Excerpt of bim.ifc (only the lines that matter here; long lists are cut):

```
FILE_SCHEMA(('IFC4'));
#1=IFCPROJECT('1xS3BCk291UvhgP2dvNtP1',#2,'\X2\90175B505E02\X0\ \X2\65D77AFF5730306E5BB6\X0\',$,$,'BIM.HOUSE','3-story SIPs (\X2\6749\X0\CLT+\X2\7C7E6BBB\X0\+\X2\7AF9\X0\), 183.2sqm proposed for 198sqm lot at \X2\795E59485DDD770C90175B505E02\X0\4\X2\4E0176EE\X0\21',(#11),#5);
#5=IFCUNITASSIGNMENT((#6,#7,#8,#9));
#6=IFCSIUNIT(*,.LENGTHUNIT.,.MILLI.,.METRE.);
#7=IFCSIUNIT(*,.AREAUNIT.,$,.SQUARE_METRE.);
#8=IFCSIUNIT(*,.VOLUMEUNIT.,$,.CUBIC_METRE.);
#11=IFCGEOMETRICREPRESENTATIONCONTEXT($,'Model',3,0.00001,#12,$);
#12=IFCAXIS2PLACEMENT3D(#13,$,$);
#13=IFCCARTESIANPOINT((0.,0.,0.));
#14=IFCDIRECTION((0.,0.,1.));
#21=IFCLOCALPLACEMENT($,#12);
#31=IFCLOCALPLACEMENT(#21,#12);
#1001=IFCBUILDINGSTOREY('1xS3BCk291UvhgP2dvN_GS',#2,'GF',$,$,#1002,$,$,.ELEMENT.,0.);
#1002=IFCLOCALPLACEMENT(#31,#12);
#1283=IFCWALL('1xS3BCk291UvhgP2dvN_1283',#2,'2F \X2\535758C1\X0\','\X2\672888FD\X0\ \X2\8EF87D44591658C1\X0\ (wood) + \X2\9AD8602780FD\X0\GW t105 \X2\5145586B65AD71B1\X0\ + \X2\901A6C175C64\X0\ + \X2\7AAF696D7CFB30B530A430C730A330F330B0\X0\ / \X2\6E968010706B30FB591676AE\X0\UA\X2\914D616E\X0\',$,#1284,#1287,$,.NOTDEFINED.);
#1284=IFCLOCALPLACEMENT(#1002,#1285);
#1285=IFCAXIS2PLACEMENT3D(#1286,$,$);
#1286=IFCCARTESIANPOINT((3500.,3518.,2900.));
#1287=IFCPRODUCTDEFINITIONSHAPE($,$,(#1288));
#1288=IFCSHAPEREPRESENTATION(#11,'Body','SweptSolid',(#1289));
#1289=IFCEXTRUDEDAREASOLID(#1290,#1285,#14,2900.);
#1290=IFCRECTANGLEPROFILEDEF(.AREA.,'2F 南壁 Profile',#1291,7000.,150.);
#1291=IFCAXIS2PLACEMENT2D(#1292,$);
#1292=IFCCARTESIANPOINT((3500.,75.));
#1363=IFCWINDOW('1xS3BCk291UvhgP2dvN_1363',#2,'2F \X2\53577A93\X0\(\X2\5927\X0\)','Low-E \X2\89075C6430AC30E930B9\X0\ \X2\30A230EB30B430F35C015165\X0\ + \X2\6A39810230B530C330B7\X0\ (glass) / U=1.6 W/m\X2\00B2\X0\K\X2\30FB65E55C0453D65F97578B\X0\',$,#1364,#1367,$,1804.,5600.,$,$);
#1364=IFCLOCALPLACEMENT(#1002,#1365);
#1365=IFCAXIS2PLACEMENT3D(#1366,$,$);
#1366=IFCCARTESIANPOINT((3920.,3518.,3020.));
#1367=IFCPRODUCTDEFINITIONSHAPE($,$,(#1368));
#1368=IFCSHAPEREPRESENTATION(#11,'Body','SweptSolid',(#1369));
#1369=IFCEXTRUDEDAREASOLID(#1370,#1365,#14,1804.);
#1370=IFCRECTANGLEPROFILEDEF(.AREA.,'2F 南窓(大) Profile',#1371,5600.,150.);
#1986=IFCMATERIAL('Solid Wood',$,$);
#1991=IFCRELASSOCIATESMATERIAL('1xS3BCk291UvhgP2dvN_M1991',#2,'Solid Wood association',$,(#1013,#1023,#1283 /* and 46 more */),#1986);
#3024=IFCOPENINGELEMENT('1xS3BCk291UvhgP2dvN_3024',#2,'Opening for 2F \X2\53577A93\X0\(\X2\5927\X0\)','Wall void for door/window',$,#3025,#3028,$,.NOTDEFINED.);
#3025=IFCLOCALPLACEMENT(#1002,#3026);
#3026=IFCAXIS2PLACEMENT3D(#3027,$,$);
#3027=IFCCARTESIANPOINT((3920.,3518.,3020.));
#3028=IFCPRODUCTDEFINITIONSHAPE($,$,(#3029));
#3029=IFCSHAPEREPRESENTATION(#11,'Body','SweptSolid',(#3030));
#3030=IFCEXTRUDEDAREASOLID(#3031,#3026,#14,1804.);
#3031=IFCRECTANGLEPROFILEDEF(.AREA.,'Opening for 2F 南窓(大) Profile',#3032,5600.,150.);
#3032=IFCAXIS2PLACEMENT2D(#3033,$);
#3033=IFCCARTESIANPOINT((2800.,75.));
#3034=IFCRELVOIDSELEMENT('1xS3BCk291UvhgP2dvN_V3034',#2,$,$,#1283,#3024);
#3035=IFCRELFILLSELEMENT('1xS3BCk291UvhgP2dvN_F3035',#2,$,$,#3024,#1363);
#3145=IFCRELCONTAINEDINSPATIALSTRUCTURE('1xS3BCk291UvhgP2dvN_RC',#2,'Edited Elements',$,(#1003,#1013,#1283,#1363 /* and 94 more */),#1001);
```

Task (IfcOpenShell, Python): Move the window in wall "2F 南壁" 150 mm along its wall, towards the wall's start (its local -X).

```python
import ifcopenshell
import ifcopenshell.api.geometry
import ifcopenshell.util.placement
import ifcopenshell.util.unit

model = ifcopenshell.open("bim.ifc")
unit_scale = ifcopenshell.util.unit.calculate_unit_scale(model)

window = model.by_guid("1xS3BCk291UvhgP2dvN_1363")
opening = window.FillsVoids[0].RelatingOpeningElement
wall = opening.VoidsElements[0].RelatingBuildingElement

wall_matrix = ifcopenshell.util.placement.get_local_placement(wall.ObjectPlacement)
shift = wall_matrix[:3, 0] * -0.15 / unit_scale
before = ifcopenshell.util.placement.get_local_placement(window.ObjectPlacement)[:3, 3].copy()

# The window is not placed relative to its opening, so move both.
for product in (opening, window):
    matrix = ifcopenshell.util.placement.get_local_placement(product.ObjectPlacement)
    matrix[:3, 3] += shift
    ifcopenshell.api.geometry.edit_object_placement(model, product=product, matrix=matrix, is_si=False)

after = ifcopenshell.util.placement.get_local_placement(window.ObjectPlacement)[:3, 3]
print("window moved by", (after - before).round(3) + 0.0)

model.write("bim_edited.ifc")
```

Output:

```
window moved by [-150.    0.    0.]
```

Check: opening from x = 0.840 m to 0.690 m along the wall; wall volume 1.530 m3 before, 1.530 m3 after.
